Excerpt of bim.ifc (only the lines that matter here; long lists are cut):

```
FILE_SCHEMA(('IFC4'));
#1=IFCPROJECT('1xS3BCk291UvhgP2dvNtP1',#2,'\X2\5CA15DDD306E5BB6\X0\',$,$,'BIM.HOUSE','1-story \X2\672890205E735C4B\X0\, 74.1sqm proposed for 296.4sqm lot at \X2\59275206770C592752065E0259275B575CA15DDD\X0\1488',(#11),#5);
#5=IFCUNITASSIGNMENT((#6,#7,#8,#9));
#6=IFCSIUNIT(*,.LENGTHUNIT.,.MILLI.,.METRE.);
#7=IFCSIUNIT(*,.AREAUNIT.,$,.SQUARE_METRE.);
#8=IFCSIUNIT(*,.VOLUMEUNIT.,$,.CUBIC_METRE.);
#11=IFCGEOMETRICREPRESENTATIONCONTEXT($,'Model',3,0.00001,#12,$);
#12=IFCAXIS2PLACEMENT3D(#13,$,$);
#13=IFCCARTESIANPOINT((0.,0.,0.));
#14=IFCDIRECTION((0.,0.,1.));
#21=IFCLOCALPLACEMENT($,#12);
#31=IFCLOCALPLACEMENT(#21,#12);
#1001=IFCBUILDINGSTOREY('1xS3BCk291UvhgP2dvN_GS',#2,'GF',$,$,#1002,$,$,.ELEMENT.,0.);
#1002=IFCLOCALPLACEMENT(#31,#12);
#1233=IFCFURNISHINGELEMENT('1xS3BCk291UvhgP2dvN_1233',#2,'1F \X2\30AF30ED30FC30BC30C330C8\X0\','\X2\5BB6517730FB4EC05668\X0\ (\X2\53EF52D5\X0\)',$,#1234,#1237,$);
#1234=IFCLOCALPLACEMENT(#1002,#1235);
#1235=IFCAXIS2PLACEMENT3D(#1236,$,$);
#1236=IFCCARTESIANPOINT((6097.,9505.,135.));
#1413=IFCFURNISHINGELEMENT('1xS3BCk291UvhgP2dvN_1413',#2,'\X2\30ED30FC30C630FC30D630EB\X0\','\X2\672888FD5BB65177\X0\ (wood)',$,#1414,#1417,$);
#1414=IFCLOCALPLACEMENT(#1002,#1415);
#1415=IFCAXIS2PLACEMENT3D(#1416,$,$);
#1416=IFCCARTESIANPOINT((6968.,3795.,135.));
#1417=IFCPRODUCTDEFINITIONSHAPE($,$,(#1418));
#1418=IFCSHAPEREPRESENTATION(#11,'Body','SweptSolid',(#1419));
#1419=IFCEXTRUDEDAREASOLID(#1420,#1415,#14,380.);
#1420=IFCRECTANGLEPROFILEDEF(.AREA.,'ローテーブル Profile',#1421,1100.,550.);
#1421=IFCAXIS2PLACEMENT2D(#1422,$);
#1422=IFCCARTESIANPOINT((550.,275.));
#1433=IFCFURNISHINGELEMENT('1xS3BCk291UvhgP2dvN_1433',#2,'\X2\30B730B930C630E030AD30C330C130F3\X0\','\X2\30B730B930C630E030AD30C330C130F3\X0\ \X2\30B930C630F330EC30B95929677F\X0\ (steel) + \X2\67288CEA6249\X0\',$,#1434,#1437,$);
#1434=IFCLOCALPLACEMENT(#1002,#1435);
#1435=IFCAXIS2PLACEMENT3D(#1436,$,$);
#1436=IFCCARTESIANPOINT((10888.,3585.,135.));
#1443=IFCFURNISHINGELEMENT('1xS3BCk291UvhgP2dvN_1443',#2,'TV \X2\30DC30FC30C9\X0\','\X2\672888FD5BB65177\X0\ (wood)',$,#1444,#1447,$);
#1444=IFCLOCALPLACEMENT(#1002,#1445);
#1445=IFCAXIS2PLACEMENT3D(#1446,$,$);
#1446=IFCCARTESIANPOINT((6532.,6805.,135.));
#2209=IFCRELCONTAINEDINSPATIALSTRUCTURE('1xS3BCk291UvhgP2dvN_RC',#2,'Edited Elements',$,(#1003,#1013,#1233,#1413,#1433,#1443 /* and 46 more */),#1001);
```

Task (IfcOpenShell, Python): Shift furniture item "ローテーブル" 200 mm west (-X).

```python
import ifcopenshell
import ifcopenshell.api.geometry
import ifcopenshell.util.placement
import ifcopenshell.util.unit

model = ifcopenshell.open("bim.ifc")
unit_scale = ifcopenshell.util.unit.calculate_unit_scale(model)

item = model.by_guid("1xS3BCk291UvhgP2dvN_1413")
matrix = ifcopenshell.util.placement.get_local_placement(item.ObjectPlacement)
matrix[0, 3] -= 0.2 / unit_scale
ifcopenshell.api.geometry.edit_object_placement(model, product=item, matrix=matrix, is_si=False)

print(ifcopenshell.util.placement.get_local_placement(item.ObjectPlacement).round(3) + 0.0)

model.write("bim_v2.ifc")
```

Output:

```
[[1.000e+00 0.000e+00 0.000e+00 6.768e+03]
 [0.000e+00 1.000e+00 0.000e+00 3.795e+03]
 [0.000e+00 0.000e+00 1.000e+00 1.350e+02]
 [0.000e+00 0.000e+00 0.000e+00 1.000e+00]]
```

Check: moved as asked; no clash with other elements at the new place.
